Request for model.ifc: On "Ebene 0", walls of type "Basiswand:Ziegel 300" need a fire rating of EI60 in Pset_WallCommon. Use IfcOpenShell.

First a look at what the model holds.

```python
import ifcopenshell
import ifcopenshell.util.element

model = ifcopenshell.open("model.ifc")
print(model.schema)
storey = next(s for s in model.by_type("IfcBuildingStorey") if s.Name == "Ebene 0")
walls = [e for e in ifcopenshell.util.element.get_decomposition(storey) if e.is_a("IfcWall")]
seen = {}
for e in walls:
    element_type = ifcopenshell.util.element.get_type(e)
    key = (element_type.Name if element_type != e and element_type else None, ifcopenshell.util.element.get_pset(e, "Pset_WallCommon", "FireRating"))
    seen[key] = seen.get(key, 0) + 1
for (name, value), count in sorted(seen.items(), key=str):
    print(count, "x", name, "|", value)
```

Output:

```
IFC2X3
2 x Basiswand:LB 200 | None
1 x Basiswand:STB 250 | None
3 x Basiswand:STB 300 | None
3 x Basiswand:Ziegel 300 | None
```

```python
import ifcopenshell
import ifcopenshell.api.pset
import ifcopenshell.util.element

model = ifcopenshell.open("model.ifc")

storey = next(s for s in model.by_type("IfcBuildingStorey") if s.Name == "Ebene 0")
walls = [e for e in ifcopenshell.util.element.get_decomposition(storey) if e.is_a("IfcWall")]

count = 0
for e in walls:
    element_type = ifcopenshell.util.element.get_type(e)
    if element_type in (None, e) or element_type.Name != "Basiswand:Ziegel 300":
        continue
    # add_pset returns the element's existing set when there is one.
    pset = ifcopenshell.api.pset.add_pset(model, product=e, name="Pset_WallCommon")
    ifcopenshell.api.pset.edit_pset(model, pset=pset, properties={"FireRating": "EI60"})
    count += 1

print(count, "walls updated")

model.write("model_edited.ifc")
```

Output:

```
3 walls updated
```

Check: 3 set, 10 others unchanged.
